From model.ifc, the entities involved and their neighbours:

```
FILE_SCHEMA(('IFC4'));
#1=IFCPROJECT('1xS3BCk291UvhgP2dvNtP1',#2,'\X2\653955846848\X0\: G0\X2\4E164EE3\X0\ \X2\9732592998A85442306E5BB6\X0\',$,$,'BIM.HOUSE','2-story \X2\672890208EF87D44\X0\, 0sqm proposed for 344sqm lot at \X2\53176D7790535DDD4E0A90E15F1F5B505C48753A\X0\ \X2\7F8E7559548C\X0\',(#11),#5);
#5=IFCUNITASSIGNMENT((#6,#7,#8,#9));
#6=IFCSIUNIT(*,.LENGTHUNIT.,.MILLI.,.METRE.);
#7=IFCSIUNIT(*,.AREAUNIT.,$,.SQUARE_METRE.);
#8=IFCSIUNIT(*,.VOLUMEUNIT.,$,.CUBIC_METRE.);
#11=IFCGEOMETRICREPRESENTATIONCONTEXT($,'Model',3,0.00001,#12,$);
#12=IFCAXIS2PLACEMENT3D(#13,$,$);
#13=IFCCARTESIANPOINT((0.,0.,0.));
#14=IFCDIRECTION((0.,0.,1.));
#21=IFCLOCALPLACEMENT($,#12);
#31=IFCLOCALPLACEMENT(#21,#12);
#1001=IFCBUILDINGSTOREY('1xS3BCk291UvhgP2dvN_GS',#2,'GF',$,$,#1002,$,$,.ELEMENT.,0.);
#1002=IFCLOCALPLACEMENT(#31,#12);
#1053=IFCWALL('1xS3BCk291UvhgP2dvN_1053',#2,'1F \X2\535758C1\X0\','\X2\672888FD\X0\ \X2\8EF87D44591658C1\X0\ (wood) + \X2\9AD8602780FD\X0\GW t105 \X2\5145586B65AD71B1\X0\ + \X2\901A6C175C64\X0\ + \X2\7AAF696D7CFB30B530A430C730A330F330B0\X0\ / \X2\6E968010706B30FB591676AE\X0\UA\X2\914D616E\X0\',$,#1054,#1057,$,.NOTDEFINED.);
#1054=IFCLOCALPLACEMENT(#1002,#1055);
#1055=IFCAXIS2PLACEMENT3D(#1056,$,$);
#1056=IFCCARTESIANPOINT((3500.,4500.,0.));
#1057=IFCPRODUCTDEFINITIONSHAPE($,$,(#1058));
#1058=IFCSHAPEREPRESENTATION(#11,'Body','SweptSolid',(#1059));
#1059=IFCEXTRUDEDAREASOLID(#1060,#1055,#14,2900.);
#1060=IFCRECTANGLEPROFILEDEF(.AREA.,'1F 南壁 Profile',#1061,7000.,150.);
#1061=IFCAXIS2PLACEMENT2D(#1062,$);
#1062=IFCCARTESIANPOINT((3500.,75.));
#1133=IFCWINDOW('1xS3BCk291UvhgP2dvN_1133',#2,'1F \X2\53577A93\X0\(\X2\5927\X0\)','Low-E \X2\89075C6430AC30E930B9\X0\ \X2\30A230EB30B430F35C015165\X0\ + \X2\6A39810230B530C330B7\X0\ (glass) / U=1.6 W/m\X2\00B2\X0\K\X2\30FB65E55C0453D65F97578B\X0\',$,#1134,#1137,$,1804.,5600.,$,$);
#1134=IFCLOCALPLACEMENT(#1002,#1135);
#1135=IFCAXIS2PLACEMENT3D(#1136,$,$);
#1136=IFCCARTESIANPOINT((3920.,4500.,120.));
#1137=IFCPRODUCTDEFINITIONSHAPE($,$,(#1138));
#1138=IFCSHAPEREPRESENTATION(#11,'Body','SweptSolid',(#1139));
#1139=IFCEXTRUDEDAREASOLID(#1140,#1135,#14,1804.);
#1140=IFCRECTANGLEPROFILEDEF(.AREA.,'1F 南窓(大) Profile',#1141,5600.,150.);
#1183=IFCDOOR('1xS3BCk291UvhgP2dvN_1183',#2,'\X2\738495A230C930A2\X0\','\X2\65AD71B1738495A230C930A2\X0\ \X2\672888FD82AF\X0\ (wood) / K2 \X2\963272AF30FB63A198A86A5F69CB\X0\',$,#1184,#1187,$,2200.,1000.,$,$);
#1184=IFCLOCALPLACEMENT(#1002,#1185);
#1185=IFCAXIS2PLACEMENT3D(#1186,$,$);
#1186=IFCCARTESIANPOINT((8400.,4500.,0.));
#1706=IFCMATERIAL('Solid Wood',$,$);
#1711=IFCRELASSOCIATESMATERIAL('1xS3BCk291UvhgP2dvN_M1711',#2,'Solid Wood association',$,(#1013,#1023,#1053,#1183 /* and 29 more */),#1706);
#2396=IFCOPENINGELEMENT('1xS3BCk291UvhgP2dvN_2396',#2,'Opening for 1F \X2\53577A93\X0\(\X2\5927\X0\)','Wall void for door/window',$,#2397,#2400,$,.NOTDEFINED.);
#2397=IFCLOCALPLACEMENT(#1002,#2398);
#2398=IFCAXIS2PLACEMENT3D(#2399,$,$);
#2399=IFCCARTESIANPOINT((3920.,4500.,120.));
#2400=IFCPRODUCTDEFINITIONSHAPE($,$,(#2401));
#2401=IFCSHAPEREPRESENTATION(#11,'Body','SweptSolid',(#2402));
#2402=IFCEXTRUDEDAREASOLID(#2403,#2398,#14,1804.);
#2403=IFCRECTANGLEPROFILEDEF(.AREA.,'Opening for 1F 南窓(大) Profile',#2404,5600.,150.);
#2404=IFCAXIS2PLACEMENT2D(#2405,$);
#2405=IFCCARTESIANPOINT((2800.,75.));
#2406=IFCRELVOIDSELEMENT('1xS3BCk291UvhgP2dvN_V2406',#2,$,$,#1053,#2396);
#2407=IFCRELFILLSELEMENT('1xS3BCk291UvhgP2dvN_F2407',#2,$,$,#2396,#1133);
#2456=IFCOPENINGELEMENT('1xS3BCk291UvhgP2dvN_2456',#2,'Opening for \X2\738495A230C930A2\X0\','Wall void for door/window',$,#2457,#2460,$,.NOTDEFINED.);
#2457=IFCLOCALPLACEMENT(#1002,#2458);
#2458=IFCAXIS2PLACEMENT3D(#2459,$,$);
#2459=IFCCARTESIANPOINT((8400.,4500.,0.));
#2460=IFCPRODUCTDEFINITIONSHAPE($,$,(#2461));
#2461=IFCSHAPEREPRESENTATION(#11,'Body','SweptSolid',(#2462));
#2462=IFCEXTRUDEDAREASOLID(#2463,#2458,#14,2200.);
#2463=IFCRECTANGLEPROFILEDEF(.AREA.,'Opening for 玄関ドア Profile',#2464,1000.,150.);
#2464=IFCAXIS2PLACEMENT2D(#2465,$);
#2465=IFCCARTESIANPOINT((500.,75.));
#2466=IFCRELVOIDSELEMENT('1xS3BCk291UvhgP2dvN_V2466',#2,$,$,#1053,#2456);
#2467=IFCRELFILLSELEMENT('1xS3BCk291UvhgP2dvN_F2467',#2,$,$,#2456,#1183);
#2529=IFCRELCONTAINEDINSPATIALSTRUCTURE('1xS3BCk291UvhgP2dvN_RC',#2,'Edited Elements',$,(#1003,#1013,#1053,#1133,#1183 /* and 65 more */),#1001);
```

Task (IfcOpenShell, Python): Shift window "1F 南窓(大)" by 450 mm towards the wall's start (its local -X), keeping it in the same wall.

```python
import ifcopenshell
import ifcopenshell.api.geometry
import ifcopenshell.util.placement
import ifcopenshell.util.unit

model = ifcopenshell.open("model.ifc")
unit_scale = ifcopenshell.util.unit.calculate_unit_scale(model)

window = model.by_id(1133)
opening = window.FillsVoids[0].RelatingOpeningElement
wall = opening.VoidsElements[0].RelatingBuildingElement

wall_matrix = ifcopenshell.util.placement.get_local_placement(wall.ObjectPlacement)
shift = wall_matrix[:3, 0] * -0.45 / unit_scale
before = ifcopenshell.util.placement.get_local_placement(window.ObjectPlacement)[:3, 3].copy()

# The window is not placed relative to its opening, so move both.
for product in (opening, window):
    matrix = ifcopenshell.util.placement.get_local_placement(product.ObjectPlacement)
    matrix[:3, 3] += shift
    ifcopenshell.api.geometry.edit_object_placement(model, product=product, matrix=matrix, is_si=False)

after = ifcopenshell.util.placement.get_local_placement(window.ObjectPlacement)[:3, 3]
print("window moved by", (after - before).round(3) + 0.0)

model.write("model-out.ifc")
```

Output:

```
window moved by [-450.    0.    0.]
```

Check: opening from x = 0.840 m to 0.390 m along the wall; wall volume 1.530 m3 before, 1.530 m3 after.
